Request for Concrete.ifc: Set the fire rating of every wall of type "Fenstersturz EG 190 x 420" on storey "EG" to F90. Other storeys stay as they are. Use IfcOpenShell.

First a look at what the model holds.

```python
import ifcopenshell
import ifcopenshell.util.element

model = ifcopenshell.open("Concrete.ifc")
print(model.schema)
storey = next(s for s in model.by_type("IfcBuildingStorey") if s.Name == "EG")
walls = [e for e in ifcopenshell.util.element.get_decomposition(storey) if e.is_a("IfcWall")]
seen = {}
for e in walls:
    element_type = ifcopenshell.util.element.get_type(e)
    key = (element_type.Name if element_type != e and element_type else None, ifcopenshell.util.element.get_pset(e, "Pset_WallCommon", "FireRating"))
    seen[key] = seen.get(key, 0) + 1
for (name, value), count in sorted(seen.items(), key=str):
    print(count, "x", name, "|", value)
```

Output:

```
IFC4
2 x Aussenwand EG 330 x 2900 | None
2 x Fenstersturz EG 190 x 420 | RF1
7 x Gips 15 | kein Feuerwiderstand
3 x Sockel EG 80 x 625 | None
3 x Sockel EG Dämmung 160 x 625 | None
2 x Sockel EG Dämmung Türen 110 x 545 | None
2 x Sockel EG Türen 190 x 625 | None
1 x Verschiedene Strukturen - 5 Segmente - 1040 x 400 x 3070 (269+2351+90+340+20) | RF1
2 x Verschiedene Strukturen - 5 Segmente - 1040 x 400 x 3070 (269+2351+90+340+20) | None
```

```python
import ifcopenshell
import ifcopenshell.api.pset
import ifcopenshell.util.element

model = ifcopenshell.open("Concrete.ifc")

storey = next(s for s in model.by_type("IfcBuildingStorey") if s.Name == "EG")
walls = [e for e in ifcopenshell.util.element.get_decomposition(storey) if e.is_a("IfcWall")]

count = 0
for e in walls:
    element_type = ifcopenshell.util.element.get_type(e)
    if element_type in (None, e) or element_type.Name != "Fenstersturz EG 190 x 420":
        continue
    # add_pset returns the element's existing set when there is one.
    pset = ifcopenshell.api.pset.add_pset(model, product=e, name="Pset_WallCommon")
    ifcopenshell.api.pset.edit_pset(model, pset=pset, properties={"FireRating": "F90"})
    count += 1

print(count, "walls updated")

model.write("Concrete_edited.ifc")
```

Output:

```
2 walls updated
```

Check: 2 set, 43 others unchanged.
